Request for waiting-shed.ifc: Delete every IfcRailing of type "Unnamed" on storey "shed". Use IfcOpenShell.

First a look at what the model holds.

```python
import ifcopenshell
import ifcopenshell.util.element

model = ifcopenshell.open("waiting-shed.ifc")
print(model.schema)
storey = next(s for s in model.by_type("IfcBuildingStorey") if s.Name == "shed")
railings = [e for e in ifcopenshell.util.element.get_decomposition(storey) if e.is_a("IfcRailing")]
seen = {}
for e in railings:
    element_type = ifcopenshell.util.element.get_type(e)
    name = element_type.Name if element_type not in (None, e) else None
    seen[name] = seen.get(name, 0) + 1
for name, count in sorted(seen.items(), key=str):
    print(count, "x", name)
```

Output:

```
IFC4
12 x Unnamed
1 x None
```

```python
import ifcopenshell
import ifcopenshell.api.root
import ifcopenshell.util.element

model = ifcopenshell.open("waiting-shed.ifc")

storey = next(s for s in model.by_type("IfcBuildingStorey") if s.Name == "shed")
railings = [e for e in ifcopenshell.util.element.get_decomposition(storey) if e.is_a("IfcRailing")]
targets = [e for e in railings if (t := ifcopenshell.util.element.get_type(e)) not in (None, e) and t.Name == "Unnamed"]

for e in targets:
    ifcopenshell.api.root.remove_product(model, product=e)
print(len(targets), "removed")

model.write("waiting-shed_v2.ifc")
```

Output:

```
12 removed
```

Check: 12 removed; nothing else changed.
